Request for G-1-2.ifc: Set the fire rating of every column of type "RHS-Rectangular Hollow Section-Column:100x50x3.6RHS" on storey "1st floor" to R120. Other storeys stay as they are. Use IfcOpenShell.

First a look at what the model holds.

```python
import ifcopenshell
import ifcopenshell.util.element

model = ifcopenshell.open("G-1-2.ifc")
print(model.schema)
storey = next(s for s in model.by_type("IfcBuildingStorey") if s.Name == "1st floor")
columns = [e for e in ifcopenshell.util.element.get_decomposition(storey) if e.is_a("IfcColumn")]
seen = {}
for e in columns:
    element_type = ifcopenshell.util.element.get_type(e)
    key = (element_type.Name if element_type != e and element_type else None, ifcopenshell.util.element.get_pset(e, "Pset_ColumnCommon", "FireRating"))
    seen[key] = seen.get(key, 0) + 1
for (name, value), count in sorted(seen.items(), key=str):
    print(count, "x", name, "|", value)
```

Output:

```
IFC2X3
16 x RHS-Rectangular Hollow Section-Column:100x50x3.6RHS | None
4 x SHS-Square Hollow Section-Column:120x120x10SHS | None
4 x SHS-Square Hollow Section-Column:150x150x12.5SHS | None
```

```python
import ifcopenshell
import ifcopenshell.api.pset
import ifcopenshell.util.element

model = ifcopenshell.open("G-1-2.ifc")

storey = next(s for s in model.by_type("IfcBuildingStorey") if s.Name == "1st floor")
columns = [e for e in ifcopenshell.util.element.get_decomposition(storey) if e.is_a("IfcColumn")]

count = 0
for e in columns:
    element_type = ifcopenshell.util.element.get_type(e)
    if element_type in (None, e) or element_type.Name != "RHS-Rectangular Hollow Section-Column:100x50x3.6RHS":
        continue
    # add_pset returns the element's existing set when there is one.
    pset = ifcopenshell.api.pset.add_pset(model, product=e, name="Pset_ColumnCommon")
    ifcopenshell.api.pset.edit_pset(model, pset=pset, properties={"FireRating": "R120"})
    count += 1

print(count, "columns updated")

model.write("G-1-2_v2.ifc")
```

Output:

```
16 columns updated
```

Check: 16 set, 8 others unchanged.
